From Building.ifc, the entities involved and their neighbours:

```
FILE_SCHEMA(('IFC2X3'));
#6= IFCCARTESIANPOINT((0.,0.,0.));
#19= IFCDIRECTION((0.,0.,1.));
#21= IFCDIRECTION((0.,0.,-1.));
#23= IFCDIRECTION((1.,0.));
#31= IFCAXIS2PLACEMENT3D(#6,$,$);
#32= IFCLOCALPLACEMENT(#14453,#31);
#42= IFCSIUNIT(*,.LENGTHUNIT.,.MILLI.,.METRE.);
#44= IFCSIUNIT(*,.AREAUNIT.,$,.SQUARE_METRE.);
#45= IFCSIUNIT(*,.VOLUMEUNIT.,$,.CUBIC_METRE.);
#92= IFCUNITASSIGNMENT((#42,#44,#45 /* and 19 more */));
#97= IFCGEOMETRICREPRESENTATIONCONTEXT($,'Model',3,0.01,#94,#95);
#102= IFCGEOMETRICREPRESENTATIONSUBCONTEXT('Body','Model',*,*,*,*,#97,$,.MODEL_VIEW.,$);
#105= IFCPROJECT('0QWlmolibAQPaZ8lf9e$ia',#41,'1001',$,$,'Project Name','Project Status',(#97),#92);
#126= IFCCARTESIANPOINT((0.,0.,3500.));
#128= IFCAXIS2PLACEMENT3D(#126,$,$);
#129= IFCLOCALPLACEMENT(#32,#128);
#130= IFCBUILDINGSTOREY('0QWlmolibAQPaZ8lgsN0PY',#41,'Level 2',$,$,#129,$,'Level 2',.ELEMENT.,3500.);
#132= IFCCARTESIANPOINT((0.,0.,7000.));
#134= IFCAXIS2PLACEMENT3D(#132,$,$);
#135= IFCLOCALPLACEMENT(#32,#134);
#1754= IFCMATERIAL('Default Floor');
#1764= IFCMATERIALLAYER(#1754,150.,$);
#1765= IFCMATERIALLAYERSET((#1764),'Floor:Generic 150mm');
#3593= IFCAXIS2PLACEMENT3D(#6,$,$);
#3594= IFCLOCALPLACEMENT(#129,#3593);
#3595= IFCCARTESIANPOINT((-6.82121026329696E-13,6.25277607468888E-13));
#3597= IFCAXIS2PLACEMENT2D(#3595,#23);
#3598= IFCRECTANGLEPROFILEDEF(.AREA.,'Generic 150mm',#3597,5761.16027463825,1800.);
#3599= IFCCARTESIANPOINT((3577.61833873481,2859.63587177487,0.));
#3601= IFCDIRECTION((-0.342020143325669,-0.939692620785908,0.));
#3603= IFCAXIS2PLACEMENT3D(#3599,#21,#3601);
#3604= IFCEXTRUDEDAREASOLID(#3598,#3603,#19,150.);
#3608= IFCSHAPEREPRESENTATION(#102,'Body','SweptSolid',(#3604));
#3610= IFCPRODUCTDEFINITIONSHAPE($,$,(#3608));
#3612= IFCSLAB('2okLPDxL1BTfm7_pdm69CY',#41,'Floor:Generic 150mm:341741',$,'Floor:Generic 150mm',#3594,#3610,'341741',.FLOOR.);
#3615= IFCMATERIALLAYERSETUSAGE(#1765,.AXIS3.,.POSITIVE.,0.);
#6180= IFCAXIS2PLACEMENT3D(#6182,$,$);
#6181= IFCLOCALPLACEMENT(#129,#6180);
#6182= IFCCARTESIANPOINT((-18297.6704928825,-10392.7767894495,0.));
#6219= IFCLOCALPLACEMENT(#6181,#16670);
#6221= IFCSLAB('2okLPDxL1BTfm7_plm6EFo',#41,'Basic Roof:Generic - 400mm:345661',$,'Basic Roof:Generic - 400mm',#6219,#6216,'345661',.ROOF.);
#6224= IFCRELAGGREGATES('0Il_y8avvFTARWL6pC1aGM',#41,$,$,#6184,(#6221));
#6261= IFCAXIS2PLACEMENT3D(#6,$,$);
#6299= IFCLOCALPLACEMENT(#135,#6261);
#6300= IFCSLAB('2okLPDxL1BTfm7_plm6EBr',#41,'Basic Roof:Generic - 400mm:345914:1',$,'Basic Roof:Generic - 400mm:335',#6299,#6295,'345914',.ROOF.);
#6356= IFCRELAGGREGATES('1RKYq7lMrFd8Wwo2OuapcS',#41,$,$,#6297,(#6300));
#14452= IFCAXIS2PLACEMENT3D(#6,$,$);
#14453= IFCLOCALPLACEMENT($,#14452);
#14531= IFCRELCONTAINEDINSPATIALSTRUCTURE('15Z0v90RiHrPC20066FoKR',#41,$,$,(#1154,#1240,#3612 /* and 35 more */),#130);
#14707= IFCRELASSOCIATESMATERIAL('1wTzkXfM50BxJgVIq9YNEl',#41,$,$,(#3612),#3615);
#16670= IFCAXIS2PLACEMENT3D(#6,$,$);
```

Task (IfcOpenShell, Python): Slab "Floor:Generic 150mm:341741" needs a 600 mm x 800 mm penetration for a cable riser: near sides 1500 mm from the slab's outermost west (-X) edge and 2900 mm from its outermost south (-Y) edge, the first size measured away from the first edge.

```python
import numpy as np
import ifcopenshell
import ifcopenshell.api.feature
import ifcopenshell.api.geometry
import ifcopenshell.api.root
import ifcopenshell.geom
import ifcopenshell.util.placement
import ifcopenshell.util.representation
import ifcopenshell.util.shape
import ifcopenshell.util.unit

model = ifcopenshell.open("Building.ifc")
unit_scale = ifcopenshell.util.unit.calculate_unit_scale(model)
settings = ifcopenshell.geom.settings()


def volume(element):
    """Net volume in cubic metres, openings subtracted."""
    shape = ifcopenshell.geom.create_shape(settings, element)
    return ifcopenshell.util.shape.get_volume(shape.geometry)


slab = model.by_id(3612)
before = volume(slab)

# Extent in the slab's own axes, in metres. The edges named are its -X and -Y sides.
slab_shape = ifcopenshell.geom.create_shape(settings, slab)
vertices = ifcopenshell.util.shape.get_vertices(slab_shape.geometry)
x_min, y_min, bottom = vertices.min(axis=0)
top = vertices[:, 2].max()

opening = ifcopenshell.api.root.create_entity(model, ifc_class="IfcOpeningElement", name="Cable riser opening")
context = ifcopenshell.util.representation.get_context(model, "Model", "Body", "MODEL_VIEW")
width, depth = 0.6, 0.8
outline = [(0.0, 0.0), (width, 0.0), (width, depth), (0.0, depth), (0.0, 0.0)]
# Overshoot both faces by 50 mm so the cut is clean.
shape = ifcopenshell.api.geometry.add_slab_representation(
    model, context=context, depth=top - bottom + 0.1, polyline=outline
)
ifcopenshell.api.geometry.assign_representation(model, product=opening, representation=shape)

matrix = ifcopenshell.util.placement.get_local_placement(slab.ObjectPlacement)
matrix[:, 3] = matrix @ np.append(np.array([x_min + 1.5, y_min + 2.9, bottom - 0.05]) / unit_scale, 1.0)
ifcopenshell.api.geometry.edit_object_placement(model, product=opening, matrix=matrix, is_si=False)
ifcopenshell.api.feature.add_feature(model, feature=opening, element=slab)

after = volume(slab)

print(f"slab volume {before:.3f} -> {after:.3f} m3")

model.write("Building_rev.ifc")
```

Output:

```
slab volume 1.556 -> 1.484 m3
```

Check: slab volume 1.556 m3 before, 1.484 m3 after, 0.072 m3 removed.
